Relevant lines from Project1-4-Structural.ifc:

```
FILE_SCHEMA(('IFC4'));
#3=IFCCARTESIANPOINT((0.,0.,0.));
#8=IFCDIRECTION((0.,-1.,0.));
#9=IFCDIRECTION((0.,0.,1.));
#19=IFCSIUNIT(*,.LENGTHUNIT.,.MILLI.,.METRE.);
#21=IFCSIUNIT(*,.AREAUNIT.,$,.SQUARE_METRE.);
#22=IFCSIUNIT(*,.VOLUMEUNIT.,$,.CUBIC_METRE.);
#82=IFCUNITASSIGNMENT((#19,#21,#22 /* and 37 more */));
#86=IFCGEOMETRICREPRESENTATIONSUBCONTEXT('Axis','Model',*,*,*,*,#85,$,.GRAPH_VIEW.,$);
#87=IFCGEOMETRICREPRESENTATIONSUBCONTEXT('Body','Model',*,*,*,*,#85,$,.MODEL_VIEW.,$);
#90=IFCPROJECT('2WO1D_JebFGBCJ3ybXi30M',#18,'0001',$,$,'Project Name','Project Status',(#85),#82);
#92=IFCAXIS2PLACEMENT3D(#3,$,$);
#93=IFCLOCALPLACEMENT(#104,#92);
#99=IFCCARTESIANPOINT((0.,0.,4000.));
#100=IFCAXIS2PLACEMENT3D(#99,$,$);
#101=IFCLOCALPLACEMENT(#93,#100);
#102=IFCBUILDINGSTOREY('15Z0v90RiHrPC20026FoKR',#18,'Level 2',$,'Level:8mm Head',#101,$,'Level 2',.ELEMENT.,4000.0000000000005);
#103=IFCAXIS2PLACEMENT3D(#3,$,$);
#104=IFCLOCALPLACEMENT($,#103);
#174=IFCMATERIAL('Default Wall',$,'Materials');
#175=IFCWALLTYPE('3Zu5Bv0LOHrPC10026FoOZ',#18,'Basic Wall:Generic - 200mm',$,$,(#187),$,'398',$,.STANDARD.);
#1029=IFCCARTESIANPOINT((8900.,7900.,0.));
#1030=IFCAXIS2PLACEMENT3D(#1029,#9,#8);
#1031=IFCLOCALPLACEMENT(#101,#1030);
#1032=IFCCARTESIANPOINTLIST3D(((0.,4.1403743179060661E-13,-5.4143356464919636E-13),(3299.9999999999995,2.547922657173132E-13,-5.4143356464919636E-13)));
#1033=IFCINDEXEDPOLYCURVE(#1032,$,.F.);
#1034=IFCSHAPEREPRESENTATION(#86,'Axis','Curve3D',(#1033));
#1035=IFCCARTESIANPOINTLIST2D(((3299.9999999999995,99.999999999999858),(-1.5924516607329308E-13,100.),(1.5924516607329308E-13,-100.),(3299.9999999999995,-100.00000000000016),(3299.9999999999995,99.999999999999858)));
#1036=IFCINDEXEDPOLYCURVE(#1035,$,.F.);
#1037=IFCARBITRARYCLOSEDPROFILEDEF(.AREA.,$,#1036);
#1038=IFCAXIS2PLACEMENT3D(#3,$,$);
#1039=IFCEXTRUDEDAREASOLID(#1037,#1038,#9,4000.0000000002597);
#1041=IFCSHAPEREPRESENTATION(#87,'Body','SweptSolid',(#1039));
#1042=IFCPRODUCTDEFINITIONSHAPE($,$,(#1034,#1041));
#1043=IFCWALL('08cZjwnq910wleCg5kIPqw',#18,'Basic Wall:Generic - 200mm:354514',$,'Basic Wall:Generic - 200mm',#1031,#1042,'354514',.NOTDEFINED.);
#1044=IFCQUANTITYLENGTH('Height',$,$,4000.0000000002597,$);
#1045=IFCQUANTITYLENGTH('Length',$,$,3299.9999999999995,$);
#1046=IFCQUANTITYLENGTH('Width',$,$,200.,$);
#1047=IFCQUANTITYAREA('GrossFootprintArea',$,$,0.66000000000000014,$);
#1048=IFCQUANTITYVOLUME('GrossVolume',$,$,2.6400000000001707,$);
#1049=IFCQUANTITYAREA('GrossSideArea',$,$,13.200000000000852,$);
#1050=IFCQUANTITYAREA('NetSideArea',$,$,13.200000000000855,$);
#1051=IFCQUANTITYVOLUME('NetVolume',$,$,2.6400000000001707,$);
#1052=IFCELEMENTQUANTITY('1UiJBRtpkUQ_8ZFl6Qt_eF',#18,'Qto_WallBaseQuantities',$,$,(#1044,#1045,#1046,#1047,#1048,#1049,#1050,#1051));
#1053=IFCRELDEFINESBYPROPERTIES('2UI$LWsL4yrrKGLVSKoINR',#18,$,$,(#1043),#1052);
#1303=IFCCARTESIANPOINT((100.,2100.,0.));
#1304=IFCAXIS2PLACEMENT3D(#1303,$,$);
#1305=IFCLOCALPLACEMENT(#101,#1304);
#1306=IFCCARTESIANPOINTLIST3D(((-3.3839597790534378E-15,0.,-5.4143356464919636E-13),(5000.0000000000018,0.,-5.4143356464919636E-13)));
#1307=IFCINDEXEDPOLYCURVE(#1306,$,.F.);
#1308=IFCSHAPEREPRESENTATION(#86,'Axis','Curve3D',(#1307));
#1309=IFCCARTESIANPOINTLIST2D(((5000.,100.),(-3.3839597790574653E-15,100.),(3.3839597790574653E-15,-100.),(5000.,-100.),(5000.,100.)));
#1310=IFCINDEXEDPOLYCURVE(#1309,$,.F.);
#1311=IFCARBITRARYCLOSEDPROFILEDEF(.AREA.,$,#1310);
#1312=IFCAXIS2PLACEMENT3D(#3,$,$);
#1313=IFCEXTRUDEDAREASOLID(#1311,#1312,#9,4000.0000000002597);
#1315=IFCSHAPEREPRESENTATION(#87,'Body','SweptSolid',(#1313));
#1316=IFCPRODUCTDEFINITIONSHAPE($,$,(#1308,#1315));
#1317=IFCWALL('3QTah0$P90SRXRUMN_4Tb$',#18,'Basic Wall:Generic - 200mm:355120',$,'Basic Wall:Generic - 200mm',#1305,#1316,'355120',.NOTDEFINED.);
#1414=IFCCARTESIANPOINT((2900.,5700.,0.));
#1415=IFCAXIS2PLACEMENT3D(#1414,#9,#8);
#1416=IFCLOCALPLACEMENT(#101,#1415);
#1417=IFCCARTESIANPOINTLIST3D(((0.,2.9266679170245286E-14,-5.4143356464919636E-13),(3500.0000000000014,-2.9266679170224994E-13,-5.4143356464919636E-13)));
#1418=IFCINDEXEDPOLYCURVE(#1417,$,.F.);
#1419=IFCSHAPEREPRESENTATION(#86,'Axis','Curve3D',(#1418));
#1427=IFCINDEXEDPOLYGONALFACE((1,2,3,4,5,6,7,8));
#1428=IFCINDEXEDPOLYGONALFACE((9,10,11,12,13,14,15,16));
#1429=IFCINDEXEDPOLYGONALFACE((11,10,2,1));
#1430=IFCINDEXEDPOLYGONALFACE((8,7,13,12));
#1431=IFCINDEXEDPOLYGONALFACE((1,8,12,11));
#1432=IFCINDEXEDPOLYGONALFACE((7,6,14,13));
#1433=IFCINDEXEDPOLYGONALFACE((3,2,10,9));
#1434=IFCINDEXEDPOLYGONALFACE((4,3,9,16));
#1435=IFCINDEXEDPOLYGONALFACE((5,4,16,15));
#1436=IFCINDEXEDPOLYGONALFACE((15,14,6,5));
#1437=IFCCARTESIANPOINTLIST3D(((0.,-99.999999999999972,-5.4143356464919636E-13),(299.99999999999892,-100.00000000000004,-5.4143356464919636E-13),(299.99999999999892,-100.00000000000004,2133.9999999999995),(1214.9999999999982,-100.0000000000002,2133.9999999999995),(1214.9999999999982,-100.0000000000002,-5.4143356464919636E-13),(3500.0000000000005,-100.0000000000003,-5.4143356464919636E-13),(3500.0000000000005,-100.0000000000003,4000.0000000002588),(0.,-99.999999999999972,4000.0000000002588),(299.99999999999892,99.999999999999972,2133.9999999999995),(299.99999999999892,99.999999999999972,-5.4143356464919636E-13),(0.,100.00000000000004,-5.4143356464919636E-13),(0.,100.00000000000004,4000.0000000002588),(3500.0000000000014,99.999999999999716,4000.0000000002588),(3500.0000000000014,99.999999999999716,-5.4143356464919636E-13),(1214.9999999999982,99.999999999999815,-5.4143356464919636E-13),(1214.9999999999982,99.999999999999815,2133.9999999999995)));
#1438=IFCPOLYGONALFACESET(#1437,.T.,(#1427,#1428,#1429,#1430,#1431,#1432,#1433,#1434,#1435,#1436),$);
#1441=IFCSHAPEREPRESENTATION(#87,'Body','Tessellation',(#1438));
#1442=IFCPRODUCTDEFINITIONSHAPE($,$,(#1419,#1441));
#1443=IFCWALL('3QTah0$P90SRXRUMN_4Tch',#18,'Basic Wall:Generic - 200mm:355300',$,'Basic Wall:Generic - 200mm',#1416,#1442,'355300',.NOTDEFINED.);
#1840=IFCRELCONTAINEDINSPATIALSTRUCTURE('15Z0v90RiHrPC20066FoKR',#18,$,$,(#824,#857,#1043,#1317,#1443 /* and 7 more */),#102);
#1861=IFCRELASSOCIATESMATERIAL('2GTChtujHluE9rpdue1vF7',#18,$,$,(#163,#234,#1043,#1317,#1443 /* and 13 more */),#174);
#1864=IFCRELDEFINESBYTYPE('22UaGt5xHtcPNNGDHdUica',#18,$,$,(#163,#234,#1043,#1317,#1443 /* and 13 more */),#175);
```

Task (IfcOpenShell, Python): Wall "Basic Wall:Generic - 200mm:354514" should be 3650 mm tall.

```python
import ifcopenshell
import ifcopenshell.api.pset
import ifcopenshell.geom
import ifcopenshell.util.element
import ifcopenshell.util.representation
import ifcopenshell.util.shape
import ifcopenshell.util.unit

model = ifcopenshell.open("Project1-4-Structural.ifc")
unit_scale = ifcopenshell.util.unit.calculate_unit_scale(model)
area_scale = ifcopenshell.util.unit.calculate_unit_scale(model, "AREAUNIT")
volume_scale = ifcopenshell.util.unit.calculate_unit_scale(model, "VOLUMEUNIT")
settings = ifcopenshell.geom.settings()


def volume(element):
    """Net volume in cubic metres, openings subtracted."""
    shape = ifcopenshell.geom.create_shape(settings, element)
    return ifcopenshell.util.shape.get_volume(shape.geometry)


wall = model.by_guid("08cZjwnq910wleCg5kIPqw")
before = volume(wall)

body = ifcopenshell.util.representation.get_representation(wall, "Model", "Body")
solid = body.Items[0]
old_height = solid.Depth
solid.Depth = 3.65 / unit_scale
after = volume(wall)
thickness = 0.2  # wall thickness in metres

# Update the stored height, areas and volumes.
qto = model.by_id(ifcopenshell.util.element.get_pset(wall, "Qto_WallBaseQuantities", should_inherit=False)["id"])
ifcopenshell.api.pset.edit_qto(model, qto=qto, properties={
    "Height": solid.Depth,
    "GrossVolume": ifcopenshell.util.element.get_pset(wall, "Qto_WallBaseQuantities", "GrossVolume") * solid.Depth / old_height,
    "GrossSideArea": ifcopenshell.util.element.get_pset(wall, "Qto_WallBaseQuantities", "GrossSideArea") * solid.Depth / old_height,
    "NetSideArea": after / thickness / area_scale,
    "NetVolume": after / volume_scale,
})

print(f"height {old_height:g} -> {solid.Depth:g}, volume {before:.3f} -> {after:.3f} m3")

model.write("Project1-4-Structural_edited.ifc")
```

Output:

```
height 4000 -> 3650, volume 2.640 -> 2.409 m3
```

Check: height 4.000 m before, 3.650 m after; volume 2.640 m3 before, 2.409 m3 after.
